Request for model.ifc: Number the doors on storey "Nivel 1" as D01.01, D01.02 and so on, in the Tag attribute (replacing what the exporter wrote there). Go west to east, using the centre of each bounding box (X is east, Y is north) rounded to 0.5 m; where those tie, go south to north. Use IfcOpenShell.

First a look at what the model holds.

```python
import ifcopenshell
import ifcopenshell.util.element
import ifcopenshell.util.placement

model = ifcopenshell.open("model.ifc")
print(model.schema)
storey = next(s for s in model.by_type("IfcBuildingStorey") if s.Name == "Nivel 1")
doors = [e for e in ifcopenshell.util.element.get_decomposition(storey) if e.is_a("IfcDoor")]
for e in sorted(doors, key=lambda e: e.id()):
    origin = ifcopenshell.util.placement.get_local_placement(e.ObjectPlacement)[:3, 3]
    print(e.id(), e.Tag, e.Name, origin.round(2) + 0.0, sep=" | ")
```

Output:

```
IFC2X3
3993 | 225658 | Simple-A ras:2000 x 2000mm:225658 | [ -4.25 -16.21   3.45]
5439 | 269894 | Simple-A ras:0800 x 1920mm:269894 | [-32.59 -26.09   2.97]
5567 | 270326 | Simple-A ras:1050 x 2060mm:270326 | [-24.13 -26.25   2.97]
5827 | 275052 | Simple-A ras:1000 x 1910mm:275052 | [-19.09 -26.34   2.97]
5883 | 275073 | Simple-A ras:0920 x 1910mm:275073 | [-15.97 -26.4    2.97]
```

```python
import ifcopenshell
import ifcopenshell.geom
import ifcopenshell.util.element
import ifcopenshell.util.shape

model = ifcopenshell.open("model.ifc")
settings = ifcopenshell.geom.settings()
settings.set("use-world-coords", True)


def centre(element):
    shape = ifcopenshell.geom.create_shape(settings, element)
    return ifcopenshell.util.shape.get_bbox_centroid(shape.geometry)


storey = next(s for s in model.by_type("IfcBuildingStorey") if s.Name == "Nivel 1")
doors = [e for e in ifcopenshell.util.element.get_decomposition(storey) if e.is_a("IfcDoor")]

# Insertion points can sit at a corner or the storey origin, so sort by the geometry (in metres).
centres = {e: centre(e) for e in doors}
doors.sort(key=lambda e: (round(centres[e][0] / 0.5), centres[e][1]))

for i, e in enumerate(doors, start=1):
    number = f"D01.{i:02d}"
    e.Tag = number
    print(e.id(), number)

model.write("model_v2.ifc")
```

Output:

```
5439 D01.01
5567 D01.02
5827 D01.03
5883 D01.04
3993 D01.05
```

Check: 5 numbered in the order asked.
